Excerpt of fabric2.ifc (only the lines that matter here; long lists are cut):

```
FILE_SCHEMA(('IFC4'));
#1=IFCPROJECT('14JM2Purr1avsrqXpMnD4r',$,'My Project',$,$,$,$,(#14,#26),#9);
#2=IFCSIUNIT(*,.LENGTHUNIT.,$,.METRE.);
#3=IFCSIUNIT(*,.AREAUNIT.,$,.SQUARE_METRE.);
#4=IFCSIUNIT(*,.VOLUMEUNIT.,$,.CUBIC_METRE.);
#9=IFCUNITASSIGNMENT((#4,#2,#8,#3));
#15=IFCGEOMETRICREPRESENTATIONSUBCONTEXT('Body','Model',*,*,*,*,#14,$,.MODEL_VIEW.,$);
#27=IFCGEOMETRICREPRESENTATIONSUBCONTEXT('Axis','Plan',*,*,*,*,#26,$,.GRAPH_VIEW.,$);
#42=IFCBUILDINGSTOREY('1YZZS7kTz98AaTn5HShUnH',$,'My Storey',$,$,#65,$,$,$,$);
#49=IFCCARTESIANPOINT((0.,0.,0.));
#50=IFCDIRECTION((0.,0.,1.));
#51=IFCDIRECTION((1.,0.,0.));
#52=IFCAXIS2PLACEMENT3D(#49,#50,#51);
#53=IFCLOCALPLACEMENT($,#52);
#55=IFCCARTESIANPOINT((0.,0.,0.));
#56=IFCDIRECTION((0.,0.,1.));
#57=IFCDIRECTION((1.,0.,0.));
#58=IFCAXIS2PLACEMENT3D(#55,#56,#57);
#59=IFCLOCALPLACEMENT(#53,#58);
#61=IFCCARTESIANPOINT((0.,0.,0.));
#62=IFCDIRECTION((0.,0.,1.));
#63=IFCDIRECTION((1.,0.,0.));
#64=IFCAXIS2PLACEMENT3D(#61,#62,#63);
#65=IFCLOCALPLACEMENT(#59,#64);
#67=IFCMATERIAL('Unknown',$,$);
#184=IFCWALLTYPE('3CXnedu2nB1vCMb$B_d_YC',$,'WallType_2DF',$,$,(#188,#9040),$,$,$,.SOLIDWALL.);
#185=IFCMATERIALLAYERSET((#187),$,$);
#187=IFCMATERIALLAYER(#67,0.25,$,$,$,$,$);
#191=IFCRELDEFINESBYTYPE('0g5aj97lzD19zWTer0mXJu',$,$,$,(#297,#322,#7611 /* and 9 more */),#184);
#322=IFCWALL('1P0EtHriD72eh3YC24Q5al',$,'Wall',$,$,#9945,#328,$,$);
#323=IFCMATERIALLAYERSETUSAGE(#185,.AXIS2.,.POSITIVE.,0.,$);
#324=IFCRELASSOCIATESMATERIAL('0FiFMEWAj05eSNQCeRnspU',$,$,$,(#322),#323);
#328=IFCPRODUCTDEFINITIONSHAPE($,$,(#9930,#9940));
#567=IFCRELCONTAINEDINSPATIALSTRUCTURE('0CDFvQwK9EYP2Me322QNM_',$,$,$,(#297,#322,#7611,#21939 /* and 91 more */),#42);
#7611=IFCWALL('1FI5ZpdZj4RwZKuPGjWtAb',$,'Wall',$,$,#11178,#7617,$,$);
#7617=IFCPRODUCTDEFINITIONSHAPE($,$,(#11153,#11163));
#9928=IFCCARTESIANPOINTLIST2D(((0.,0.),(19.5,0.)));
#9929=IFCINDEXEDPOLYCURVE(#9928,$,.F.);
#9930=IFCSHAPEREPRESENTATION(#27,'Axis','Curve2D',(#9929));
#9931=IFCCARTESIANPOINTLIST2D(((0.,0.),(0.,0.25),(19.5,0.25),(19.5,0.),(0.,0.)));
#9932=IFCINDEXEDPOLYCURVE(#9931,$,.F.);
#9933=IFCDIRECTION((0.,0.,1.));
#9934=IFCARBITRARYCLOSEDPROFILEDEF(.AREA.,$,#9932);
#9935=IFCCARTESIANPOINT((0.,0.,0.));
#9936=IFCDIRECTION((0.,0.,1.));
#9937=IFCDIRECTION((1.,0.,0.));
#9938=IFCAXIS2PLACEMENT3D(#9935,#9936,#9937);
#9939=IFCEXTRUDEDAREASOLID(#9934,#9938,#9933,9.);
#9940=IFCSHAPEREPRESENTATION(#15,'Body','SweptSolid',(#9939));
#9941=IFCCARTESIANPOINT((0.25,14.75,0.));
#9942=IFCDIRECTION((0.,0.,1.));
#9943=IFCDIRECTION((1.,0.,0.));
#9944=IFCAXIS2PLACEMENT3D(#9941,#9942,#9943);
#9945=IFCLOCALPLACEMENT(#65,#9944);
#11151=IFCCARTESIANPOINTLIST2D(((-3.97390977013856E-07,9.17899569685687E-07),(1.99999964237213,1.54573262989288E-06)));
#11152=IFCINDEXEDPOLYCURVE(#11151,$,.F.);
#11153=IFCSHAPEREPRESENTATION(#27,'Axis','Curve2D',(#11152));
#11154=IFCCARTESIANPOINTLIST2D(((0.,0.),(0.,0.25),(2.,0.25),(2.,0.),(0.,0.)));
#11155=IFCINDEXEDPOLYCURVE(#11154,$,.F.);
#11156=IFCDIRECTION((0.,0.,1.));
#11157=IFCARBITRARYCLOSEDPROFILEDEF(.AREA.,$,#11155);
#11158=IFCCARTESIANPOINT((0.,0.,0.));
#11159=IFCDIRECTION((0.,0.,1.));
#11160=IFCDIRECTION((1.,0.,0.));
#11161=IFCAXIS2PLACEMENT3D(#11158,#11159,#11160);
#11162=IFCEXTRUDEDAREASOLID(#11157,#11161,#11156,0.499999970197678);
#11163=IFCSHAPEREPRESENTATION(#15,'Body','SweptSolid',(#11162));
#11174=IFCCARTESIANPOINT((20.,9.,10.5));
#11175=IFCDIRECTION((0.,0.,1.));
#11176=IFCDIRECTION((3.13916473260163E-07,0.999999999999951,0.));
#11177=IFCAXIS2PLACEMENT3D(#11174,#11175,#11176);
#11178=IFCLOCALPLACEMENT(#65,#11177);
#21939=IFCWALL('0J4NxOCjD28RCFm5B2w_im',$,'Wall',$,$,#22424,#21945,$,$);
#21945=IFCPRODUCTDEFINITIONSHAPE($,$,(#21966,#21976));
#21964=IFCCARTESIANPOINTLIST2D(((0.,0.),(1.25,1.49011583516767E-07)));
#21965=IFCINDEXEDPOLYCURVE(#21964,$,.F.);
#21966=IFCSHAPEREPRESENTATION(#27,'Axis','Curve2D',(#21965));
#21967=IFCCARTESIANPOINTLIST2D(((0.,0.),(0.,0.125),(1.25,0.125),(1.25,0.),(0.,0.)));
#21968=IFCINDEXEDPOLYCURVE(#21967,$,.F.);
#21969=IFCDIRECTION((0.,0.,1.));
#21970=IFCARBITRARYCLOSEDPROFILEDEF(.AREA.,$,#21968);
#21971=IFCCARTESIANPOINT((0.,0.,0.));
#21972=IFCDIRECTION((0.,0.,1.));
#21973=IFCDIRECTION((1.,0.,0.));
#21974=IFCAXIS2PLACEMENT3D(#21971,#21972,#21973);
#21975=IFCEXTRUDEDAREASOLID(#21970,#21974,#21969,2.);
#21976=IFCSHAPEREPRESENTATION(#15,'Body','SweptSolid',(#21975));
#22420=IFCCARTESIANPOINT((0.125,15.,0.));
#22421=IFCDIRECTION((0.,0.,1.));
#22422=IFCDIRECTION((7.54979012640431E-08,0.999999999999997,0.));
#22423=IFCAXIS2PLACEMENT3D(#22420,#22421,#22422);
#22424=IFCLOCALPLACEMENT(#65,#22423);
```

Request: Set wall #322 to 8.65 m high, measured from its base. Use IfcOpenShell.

```python
import ifcopenshell
import ifcopenshell.geom
import ifcopenshell.util.representation
import ifcopenshell.util.shape

model = ifcopenshell.open("fabric2.ifc")
settings = ifcopenshell.geom.settings()


def volume(element):
    """Net volume in cubic metres, openings subtracted."""
    shape = ifcopenshell.geom.create_shape(settings, element)
    return ifcopenshell.util.shape.get_volume(shape.geometry)


wall = model.by_guid("1P0EtHriD72eh3YC24Q5al")
before = volume(wall)

body = ifcopenshell.util.representation.get_representation(wall, "Model", "Body")
solid = body.Items[0]
old_height = solid.Depth
solid.Depth = 8.65
after = volume(wall)

print(f"height {old_height:g} -> {solid.Depth:g}, volume {before:.3f} -> {after:.3f} m3")

model.write("fabric2_edited.ifc")
```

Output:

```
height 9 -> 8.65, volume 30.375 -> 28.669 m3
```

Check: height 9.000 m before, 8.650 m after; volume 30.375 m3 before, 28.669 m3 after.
